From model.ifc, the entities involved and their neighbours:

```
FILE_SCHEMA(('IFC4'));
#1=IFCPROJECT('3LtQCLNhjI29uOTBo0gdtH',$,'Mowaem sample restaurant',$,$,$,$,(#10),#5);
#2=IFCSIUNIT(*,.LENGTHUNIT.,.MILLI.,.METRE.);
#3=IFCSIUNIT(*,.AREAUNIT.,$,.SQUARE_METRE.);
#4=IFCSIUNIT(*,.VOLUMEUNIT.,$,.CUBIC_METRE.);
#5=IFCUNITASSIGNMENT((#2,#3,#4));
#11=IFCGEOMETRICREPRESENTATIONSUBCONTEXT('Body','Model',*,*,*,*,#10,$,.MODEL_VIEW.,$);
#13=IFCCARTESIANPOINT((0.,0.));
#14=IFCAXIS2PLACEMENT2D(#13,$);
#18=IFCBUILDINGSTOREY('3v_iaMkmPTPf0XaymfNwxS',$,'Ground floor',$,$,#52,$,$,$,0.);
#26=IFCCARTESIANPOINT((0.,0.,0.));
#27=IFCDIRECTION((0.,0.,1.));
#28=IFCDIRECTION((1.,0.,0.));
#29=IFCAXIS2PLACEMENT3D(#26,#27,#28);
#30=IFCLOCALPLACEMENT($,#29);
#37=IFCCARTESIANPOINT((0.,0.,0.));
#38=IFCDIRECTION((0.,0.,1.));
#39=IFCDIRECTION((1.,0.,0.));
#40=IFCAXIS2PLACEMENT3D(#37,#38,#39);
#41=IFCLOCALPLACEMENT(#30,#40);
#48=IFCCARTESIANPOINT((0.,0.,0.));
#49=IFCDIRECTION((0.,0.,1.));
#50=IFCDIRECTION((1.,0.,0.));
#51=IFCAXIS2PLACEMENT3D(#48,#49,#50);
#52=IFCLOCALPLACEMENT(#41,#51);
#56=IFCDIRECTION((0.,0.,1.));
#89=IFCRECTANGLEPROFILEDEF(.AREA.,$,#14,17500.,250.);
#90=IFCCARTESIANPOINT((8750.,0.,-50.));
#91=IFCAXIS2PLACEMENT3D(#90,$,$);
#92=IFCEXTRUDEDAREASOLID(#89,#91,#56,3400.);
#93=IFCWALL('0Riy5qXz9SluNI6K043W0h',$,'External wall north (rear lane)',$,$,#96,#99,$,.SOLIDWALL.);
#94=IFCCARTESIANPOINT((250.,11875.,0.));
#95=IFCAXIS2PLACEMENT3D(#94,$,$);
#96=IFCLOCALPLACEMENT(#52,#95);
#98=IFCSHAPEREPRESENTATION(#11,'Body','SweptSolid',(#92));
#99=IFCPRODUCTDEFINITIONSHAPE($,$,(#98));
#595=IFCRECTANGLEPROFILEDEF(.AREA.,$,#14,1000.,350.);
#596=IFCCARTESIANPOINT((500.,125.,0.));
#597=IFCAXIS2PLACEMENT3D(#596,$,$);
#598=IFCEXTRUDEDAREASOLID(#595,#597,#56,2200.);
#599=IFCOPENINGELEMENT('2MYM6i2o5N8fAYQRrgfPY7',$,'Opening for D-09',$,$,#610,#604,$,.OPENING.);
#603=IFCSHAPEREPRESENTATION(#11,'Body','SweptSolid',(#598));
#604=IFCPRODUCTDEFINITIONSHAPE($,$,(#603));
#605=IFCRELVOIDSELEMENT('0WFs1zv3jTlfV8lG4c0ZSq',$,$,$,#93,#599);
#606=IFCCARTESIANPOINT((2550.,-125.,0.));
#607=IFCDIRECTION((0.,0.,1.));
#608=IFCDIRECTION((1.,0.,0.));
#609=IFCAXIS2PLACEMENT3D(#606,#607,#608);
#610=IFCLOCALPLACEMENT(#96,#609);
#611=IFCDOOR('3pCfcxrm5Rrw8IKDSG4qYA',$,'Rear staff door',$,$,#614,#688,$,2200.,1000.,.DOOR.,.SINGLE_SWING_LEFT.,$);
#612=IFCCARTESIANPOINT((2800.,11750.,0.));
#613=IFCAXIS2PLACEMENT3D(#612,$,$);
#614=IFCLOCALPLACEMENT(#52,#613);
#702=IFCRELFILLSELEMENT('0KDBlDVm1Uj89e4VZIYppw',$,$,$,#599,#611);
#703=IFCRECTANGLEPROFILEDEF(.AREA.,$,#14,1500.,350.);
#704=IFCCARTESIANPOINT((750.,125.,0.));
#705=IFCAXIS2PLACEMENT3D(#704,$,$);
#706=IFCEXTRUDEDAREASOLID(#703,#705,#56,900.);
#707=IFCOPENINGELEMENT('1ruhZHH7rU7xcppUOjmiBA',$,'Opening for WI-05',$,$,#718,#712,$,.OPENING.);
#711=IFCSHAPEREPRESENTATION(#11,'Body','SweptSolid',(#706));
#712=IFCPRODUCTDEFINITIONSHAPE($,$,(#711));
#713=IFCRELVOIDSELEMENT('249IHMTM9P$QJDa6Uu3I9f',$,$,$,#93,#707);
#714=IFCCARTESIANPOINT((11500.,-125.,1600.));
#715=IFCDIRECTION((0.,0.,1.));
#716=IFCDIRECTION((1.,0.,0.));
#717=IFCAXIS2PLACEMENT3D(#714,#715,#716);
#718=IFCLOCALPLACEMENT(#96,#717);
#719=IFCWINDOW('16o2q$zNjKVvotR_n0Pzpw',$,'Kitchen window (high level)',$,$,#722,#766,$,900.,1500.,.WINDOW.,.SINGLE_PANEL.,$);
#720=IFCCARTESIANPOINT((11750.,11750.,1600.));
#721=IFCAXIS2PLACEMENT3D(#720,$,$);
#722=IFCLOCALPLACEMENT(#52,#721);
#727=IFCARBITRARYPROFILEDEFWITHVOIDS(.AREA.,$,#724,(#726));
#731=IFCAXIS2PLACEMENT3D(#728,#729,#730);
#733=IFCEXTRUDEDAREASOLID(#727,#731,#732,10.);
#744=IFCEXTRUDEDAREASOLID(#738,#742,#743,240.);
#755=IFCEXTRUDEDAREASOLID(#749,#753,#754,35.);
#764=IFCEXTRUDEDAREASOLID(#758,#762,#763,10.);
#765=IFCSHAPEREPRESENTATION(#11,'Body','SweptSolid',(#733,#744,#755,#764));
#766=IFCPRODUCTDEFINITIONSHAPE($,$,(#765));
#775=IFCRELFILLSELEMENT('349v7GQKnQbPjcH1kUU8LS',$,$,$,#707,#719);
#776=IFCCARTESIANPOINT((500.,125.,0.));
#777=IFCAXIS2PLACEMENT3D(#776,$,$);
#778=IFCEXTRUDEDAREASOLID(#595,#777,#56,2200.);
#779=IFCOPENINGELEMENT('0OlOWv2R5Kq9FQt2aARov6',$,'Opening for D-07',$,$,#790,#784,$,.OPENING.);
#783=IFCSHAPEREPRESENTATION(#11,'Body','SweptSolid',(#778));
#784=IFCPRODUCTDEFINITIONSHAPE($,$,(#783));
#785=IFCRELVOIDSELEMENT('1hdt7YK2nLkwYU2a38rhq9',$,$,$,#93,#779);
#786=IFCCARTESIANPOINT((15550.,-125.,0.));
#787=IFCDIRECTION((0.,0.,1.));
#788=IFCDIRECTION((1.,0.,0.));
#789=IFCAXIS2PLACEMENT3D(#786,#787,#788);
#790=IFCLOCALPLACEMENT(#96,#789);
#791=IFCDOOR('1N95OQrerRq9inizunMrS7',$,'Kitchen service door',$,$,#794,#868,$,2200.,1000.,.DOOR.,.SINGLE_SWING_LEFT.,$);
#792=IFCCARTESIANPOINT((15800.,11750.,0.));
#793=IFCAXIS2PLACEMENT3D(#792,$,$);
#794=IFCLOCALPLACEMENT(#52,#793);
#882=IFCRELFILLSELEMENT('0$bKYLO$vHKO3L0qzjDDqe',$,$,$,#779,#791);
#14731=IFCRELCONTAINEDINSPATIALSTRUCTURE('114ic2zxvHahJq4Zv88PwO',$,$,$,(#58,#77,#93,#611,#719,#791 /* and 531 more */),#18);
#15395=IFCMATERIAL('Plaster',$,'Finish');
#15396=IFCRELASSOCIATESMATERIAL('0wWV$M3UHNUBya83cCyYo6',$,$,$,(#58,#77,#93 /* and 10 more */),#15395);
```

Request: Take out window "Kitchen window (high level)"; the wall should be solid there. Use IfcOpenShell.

```python
import ifcopenshell
import ifcopenshell.api.feature
import ifcopenshell.api.root
import ifcopenshell.geom
import ifcopenshell.util.shape

model = ifcopenshell.open("model.ifc")
settings = ifcopenshell.geom.settings()


def volume(element):
    """Net volume in cubic metres, openings subtracted."""
    shape = ifcopenshell.geom.create_shape(settings, element)
    return ifcopenshell.util.shape.get_volume(shape.geometry)


window = model.by_guid("16o2q$zNjKVvotR_n0Pzpw")
opening = window.FillsVoids[0].RelatingOpeningElement
wall = opening.VoidsElements[0].RelatingBuildingElement
before = volume(wall)

ifcopenshell.api.root.remove_product(model, product=window)
ifcopenshell.api.feature.remove_feature(model, feature=opening)

after = volume(wall)

print(f"wall volume {before:.3f} -> {after:.3f} m3")

model.write("model_updated.ifc")
```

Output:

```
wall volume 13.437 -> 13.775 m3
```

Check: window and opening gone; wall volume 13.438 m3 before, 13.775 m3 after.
